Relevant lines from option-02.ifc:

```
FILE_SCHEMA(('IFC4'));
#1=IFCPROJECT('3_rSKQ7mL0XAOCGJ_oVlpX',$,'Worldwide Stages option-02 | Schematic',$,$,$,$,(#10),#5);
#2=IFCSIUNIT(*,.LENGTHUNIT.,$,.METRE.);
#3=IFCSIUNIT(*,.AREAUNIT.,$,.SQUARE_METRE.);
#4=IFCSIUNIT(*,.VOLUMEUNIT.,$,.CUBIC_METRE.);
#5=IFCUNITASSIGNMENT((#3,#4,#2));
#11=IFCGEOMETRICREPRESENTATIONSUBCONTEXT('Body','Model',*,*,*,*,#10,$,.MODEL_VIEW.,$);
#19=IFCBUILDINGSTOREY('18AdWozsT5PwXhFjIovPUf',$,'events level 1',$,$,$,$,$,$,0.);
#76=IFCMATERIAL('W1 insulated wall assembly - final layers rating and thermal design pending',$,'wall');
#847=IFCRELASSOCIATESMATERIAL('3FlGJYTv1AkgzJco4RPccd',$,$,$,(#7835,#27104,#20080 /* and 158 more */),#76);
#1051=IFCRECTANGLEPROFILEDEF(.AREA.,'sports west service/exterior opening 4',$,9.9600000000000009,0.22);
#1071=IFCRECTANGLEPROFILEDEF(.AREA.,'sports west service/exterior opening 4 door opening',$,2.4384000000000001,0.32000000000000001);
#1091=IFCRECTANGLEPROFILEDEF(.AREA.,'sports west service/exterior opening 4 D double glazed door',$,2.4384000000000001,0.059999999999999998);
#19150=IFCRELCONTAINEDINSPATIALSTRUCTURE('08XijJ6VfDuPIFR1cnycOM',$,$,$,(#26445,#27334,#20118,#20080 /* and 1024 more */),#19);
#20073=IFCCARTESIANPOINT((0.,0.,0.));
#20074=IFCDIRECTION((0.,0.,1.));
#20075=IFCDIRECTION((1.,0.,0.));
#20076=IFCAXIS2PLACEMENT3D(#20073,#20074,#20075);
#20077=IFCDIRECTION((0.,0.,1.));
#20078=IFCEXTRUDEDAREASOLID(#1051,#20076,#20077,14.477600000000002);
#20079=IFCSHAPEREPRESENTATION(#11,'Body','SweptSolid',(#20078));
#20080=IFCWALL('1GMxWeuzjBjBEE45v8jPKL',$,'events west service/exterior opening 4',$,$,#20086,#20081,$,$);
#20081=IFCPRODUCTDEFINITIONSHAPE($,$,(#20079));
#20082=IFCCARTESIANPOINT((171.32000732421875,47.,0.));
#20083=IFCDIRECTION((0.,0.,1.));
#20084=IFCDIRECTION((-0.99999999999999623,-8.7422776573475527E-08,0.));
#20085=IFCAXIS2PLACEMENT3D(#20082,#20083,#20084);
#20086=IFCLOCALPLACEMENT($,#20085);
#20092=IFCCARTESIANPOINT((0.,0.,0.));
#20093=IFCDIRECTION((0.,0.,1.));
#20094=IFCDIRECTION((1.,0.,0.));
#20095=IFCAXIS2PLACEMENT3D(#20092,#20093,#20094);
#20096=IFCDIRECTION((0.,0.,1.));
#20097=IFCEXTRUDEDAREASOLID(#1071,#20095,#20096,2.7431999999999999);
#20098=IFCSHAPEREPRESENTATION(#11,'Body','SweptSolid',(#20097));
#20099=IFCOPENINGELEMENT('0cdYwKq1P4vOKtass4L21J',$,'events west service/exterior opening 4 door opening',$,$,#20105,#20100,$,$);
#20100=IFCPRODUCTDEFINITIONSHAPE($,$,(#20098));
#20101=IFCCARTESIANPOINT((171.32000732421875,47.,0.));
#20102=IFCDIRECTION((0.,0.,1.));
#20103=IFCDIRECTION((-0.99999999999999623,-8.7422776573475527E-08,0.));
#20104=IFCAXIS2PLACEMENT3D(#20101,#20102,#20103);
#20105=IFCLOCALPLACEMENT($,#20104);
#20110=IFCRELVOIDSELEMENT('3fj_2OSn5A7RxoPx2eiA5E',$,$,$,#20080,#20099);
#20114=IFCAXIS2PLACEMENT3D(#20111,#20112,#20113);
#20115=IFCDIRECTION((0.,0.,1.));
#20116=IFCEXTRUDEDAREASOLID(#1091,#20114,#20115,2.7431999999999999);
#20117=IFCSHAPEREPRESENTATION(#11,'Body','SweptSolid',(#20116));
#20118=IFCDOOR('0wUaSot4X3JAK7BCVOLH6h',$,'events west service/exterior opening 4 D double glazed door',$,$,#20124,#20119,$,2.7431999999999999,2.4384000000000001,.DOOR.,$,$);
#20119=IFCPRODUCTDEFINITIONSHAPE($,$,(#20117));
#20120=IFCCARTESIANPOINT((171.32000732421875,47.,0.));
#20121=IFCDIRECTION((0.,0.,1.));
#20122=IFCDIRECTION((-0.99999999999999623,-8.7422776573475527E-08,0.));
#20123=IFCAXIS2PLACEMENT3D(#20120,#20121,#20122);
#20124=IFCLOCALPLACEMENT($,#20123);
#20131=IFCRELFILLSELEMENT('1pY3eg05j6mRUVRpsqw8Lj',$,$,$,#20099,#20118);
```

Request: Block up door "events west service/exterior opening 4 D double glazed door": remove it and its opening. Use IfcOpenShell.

```python
import ifcopenshell
import ifcopenshell.api.feature
import ifcopenshell.api.root
import ifcopenshell.geom
import ifcopenshell.util.shape

model = ifcopenshell.open("option-02.ifc")
settings = ifcopenshell.geom.settings()


def volume(element):
    """Net volume in cubic metres, openings subtracted."""
    shape = ifcopenshell.geom.create_shape(settings, element)
    return ifcopenshell.util.shape.get_volume(shape.geometry)


door = model.by_id(20118)
opening = door.FillsVoids[0].RelatingOpeningElement
wall = opening.VoidsElements[0].RelatingBuildingElement
before = volume(wall)

ifcopenshell.api.root.remove_product(model, product=door)
ifcopenshell.api.feature.remove_feature(model, feature=opening)

after = volume(wall)

print(f"wall volume {before:.3f} -> {after:.3f} m3")

model.write("option-02_edited.ifc")
```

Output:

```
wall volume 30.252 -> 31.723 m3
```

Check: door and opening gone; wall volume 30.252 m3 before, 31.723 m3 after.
